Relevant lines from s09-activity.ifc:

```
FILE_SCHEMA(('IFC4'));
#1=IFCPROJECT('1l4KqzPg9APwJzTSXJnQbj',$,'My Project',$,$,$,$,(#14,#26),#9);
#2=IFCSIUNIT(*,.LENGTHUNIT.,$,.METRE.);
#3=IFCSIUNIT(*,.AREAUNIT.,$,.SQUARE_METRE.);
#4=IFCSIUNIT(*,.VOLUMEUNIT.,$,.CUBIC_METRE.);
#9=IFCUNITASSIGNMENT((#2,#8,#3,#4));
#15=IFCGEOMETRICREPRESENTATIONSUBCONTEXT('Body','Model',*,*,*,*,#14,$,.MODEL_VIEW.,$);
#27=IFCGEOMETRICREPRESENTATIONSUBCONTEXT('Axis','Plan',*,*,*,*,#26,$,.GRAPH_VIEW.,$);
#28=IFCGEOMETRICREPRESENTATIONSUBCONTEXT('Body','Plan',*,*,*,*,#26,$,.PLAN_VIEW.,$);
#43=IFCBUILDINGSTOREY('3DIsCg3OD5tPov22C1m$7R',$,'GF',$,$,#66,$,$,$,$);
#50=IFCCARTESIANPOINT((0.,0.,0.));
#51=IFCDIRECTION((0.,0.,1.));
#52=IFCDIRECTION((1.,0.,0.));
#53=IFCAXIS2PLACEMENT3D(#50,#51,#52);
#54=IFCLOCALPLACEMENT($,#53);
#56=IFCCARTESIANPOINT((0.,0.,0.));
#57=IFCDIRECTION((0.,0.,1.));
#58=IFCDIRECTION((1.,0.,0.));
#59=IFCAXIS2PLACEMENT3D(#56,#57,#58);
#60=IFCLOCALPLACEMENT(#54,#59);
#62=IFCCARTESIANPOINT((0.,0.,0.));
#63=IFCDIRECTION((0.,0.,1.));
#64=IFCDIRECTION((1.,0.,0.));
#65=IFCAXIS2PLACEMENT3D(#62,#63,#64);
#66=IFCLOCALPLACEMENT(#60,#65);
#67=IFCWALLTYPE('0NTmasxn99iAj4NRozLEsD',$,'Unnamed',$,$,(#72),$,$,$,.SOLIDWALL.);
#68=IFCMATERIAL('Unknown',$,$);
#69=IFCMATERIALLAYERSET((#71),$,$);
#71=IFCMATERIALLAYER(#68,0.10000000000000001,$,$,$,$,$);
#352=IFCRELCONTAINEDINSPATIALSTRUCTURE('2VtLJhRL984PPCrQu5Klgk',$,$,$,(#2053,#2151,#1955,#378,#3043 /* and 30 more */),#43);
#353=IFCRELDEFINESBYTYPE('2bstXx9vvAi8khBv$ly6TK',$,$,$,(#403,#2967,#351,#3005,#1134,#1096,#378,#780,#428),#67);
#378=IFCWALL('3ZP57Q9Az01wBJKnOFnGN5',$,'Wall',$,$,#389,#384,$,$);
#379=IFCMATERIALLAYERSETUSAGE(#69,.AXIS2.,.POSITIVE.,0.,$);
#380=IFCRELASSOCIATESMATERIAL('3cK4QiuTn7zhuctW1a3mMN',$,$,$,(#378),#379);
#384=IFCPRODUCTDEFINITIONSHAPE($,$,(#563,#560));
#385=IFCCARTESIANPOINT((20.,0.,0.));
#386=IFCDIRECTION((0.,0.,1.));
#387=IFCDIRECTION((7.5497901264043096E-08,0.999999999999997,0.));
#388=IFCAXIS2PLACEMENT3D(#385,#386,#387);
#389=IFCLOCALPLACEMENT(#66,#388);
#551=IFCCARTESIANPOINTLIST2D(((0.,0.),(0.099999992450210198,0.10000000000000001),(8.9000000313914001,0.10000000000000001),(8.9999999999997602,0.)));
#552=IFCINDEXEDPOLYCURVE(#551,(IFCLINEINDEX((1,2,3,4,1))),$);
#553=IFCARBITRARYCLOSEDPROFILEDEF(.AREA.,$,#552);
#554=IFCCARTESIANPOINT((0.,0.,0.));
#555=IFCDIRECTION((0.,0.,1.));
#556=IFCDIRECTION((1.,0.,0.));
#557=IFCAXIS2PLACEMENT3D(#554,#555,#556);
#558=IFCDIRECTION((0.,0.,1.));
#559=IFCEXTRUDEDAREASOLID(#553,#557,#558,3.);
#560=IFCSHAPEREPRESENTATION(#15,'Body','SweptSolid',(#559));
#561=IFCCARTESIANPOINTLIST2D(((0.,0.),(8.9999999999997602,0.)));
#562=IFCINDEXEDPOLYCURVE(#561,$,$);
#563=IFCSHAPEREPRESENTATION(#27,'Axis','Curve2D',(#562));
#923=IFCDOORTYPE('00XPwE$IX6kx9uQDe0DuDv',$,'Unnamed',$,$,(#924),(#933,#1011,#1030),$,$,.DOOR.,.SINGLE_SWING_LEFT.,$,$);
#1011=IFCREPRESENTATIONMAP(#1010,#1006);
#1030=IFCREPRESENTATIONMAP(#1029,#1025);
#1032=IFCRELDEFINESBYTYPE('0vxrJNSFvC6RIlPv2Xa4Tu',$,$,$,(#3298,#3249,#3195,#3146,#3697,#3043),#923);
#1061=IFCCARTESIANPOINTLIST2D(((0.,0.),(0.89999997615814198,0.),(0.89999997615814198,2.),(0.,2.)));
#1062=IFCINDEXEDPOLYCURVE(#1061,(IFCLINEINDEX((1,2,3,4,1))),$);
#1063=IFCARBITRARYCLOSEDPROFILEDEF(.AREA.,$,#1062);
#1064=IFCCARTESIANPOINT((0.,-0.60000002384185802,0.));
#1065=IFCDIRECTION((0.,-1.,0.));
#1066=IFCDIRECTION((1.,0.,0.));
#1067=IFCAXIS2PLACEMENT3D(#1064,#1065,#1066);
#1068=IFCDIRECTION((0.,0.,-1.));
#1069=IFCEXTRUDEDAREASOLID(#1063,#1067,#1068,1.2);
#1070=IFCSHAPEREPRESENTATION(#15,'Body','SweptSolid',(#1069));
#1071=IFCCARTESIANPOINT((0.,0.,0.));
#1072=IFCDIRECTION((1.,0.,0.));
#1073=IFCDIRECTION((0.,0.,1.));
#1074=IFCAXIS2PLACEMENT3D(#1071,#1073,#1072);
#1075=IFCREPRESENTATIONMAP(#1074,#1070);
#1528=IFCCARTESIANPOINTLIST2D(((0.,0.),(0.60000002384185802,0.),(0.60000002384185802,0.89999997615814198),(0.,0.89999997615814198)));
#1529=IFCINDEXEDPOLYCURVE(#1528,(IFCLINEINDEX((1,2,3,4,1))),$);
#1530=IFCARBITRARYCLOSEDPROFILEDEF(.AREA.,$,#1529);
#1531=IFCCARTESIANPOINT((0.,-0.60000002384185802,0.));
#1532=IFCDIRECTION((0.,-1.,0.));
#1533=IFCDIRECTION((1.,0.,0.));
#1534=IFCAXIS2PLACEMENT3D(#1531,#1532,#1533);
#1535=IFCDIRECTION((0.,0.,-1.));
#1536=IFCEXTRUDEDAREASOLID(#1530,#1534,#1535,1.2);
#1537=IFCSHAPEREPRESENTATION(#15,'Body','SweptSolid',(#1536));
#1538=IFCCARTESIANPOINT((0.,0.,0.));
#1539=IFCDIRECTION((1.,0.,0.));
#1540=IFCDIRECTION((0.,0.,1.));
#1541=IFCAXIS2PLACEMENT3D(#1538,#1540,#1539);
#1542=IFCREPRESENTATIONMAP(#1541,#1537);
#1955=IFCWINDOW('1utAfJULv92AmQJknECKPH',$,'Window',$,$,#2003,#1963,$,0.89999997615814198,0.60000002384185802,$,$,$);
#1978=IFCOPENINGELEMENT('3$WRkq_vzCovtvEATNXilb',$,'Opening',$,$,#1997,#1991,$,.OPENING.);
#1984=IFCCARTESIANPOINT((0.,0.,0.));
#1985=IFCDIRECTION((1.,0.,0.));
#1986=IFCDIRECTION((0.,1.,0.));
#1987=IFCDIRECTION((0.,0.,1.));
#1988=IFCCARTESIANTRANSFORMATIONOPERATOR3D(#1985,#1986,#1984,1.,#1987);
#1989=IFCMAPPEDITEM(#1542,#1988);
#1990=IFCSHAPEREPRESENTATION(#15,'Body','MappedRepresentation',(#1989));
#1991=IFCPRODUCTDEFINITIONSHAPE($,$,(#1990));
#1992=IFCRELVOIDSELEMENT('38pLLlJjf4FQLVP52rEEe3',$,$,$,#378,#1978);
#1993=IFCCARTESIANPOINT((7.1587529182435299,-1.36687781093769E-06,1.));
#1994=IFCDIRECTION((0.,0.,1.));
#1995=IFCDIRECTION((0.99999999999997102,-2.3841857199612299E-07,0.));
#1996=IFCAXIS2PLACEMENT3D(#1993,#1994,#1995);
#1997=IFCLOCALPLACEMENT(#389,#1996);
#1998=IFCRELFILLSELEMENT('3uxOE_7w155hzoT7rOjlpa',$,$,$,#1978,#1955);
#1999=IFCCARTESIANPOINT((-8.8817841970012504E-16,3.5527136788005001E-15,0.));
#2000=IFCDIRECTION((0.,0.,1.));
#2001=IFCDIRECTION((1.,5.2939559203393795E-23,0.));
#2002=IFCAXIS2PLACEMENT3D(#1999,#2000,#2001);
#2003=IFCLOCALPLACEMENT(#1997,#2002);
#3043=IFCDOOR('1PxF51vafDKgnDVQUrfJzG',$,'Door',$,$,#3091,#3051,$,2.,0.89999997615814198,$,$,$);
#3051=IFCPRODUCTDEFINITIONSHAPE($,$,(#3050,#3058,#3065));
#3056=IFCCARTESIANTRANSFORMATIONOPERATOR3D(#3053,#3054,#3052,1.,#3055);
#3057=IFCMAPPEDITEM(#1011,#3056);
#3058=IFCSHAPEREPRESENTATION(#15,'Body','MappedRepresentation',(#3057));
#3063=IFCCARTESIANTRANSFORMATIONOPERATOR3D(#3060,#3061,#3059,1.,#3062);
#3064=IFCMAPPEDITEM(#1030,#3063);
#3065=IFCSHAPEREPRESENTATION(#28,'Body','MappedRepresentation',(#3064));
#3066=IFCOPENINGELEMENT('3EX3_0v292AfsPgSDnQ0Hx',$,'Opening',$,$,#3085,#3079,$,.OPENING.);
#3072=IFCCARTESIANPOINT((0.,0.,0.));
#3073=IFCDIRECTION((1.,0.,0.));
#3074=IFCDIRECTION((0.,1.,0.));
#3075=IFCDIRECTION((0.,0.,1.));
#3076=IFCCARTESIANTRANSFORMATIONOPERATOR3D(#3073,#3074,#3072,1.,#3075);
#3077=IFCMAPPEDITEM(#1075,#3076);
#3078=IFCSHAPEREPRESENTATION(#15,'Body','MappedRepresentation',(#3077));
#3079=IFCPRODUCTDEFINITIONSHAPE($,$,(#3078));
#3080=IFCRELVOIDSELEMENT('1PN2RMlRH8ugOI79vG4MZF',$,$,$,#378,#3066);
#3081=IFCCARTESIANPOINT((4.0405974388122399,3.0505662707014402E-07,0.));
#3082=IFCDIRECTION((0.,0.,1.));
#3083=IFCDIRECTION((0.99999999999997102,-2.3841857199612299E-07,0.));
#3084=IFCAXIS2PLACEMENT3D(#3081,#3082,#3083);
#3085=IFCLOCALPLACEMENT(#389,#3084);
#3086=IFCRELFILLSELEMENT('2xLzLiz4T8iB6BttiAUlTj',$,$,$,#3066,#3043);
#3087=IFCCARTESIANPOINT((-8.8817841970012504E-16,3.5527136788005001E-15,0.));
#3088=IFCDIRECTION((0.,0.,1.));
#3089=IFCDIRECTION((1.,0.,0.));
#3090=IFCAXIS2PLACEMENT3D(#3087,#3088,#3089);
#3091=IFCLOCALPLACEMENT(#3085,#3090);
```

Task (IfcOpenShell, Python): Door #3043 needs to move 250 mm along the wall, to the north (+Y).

```python
import ifcopenshell
import ifcopenshell.api.geometry
import ifcopenshell.util.placement

model = ifcopenshell.open("s09-activity.ifc")

door = model.by_guid("1PxF51vafDKgnDVQUrfJzG")
opening = door.FillsVoids[0].RelatingOpeningElement
wall = opening.VoidsElements[0].RelatingBuildingElement

wall_matrix = ifcopenshell.util.placement.get_local_placement(wall.ObjectPlacement)
shift = wall_matrix[:3, 0] * 0.25
before = ifcopenshell.util.placement.get_local_placement(door.ObjectPlacement)[:3, 3].copy()

# The door is placed relative to its opening, so it follows when the opening moves.
matrix = ifcopenshell.util.placement.get_local_placement(opening.ObjectPlacement)
matrix[:3, 3] += shift
ifcopenshell.api.geometry.edit_object_placement(
    model, product=opening, matrix=matrix, is_si=False, should_transform_children=True
)

after = ifcopenshell.util.placement.get_local_placement(door.ObjectPlacement)[:3, 3]
print("door moved by", (after - before).round(3) + 0.0)

model.write("s09-activity-out.ifc")
```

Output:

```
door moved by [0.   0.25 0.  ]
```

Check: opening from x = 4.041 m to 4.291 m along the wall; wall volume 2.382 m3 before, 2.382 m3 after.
